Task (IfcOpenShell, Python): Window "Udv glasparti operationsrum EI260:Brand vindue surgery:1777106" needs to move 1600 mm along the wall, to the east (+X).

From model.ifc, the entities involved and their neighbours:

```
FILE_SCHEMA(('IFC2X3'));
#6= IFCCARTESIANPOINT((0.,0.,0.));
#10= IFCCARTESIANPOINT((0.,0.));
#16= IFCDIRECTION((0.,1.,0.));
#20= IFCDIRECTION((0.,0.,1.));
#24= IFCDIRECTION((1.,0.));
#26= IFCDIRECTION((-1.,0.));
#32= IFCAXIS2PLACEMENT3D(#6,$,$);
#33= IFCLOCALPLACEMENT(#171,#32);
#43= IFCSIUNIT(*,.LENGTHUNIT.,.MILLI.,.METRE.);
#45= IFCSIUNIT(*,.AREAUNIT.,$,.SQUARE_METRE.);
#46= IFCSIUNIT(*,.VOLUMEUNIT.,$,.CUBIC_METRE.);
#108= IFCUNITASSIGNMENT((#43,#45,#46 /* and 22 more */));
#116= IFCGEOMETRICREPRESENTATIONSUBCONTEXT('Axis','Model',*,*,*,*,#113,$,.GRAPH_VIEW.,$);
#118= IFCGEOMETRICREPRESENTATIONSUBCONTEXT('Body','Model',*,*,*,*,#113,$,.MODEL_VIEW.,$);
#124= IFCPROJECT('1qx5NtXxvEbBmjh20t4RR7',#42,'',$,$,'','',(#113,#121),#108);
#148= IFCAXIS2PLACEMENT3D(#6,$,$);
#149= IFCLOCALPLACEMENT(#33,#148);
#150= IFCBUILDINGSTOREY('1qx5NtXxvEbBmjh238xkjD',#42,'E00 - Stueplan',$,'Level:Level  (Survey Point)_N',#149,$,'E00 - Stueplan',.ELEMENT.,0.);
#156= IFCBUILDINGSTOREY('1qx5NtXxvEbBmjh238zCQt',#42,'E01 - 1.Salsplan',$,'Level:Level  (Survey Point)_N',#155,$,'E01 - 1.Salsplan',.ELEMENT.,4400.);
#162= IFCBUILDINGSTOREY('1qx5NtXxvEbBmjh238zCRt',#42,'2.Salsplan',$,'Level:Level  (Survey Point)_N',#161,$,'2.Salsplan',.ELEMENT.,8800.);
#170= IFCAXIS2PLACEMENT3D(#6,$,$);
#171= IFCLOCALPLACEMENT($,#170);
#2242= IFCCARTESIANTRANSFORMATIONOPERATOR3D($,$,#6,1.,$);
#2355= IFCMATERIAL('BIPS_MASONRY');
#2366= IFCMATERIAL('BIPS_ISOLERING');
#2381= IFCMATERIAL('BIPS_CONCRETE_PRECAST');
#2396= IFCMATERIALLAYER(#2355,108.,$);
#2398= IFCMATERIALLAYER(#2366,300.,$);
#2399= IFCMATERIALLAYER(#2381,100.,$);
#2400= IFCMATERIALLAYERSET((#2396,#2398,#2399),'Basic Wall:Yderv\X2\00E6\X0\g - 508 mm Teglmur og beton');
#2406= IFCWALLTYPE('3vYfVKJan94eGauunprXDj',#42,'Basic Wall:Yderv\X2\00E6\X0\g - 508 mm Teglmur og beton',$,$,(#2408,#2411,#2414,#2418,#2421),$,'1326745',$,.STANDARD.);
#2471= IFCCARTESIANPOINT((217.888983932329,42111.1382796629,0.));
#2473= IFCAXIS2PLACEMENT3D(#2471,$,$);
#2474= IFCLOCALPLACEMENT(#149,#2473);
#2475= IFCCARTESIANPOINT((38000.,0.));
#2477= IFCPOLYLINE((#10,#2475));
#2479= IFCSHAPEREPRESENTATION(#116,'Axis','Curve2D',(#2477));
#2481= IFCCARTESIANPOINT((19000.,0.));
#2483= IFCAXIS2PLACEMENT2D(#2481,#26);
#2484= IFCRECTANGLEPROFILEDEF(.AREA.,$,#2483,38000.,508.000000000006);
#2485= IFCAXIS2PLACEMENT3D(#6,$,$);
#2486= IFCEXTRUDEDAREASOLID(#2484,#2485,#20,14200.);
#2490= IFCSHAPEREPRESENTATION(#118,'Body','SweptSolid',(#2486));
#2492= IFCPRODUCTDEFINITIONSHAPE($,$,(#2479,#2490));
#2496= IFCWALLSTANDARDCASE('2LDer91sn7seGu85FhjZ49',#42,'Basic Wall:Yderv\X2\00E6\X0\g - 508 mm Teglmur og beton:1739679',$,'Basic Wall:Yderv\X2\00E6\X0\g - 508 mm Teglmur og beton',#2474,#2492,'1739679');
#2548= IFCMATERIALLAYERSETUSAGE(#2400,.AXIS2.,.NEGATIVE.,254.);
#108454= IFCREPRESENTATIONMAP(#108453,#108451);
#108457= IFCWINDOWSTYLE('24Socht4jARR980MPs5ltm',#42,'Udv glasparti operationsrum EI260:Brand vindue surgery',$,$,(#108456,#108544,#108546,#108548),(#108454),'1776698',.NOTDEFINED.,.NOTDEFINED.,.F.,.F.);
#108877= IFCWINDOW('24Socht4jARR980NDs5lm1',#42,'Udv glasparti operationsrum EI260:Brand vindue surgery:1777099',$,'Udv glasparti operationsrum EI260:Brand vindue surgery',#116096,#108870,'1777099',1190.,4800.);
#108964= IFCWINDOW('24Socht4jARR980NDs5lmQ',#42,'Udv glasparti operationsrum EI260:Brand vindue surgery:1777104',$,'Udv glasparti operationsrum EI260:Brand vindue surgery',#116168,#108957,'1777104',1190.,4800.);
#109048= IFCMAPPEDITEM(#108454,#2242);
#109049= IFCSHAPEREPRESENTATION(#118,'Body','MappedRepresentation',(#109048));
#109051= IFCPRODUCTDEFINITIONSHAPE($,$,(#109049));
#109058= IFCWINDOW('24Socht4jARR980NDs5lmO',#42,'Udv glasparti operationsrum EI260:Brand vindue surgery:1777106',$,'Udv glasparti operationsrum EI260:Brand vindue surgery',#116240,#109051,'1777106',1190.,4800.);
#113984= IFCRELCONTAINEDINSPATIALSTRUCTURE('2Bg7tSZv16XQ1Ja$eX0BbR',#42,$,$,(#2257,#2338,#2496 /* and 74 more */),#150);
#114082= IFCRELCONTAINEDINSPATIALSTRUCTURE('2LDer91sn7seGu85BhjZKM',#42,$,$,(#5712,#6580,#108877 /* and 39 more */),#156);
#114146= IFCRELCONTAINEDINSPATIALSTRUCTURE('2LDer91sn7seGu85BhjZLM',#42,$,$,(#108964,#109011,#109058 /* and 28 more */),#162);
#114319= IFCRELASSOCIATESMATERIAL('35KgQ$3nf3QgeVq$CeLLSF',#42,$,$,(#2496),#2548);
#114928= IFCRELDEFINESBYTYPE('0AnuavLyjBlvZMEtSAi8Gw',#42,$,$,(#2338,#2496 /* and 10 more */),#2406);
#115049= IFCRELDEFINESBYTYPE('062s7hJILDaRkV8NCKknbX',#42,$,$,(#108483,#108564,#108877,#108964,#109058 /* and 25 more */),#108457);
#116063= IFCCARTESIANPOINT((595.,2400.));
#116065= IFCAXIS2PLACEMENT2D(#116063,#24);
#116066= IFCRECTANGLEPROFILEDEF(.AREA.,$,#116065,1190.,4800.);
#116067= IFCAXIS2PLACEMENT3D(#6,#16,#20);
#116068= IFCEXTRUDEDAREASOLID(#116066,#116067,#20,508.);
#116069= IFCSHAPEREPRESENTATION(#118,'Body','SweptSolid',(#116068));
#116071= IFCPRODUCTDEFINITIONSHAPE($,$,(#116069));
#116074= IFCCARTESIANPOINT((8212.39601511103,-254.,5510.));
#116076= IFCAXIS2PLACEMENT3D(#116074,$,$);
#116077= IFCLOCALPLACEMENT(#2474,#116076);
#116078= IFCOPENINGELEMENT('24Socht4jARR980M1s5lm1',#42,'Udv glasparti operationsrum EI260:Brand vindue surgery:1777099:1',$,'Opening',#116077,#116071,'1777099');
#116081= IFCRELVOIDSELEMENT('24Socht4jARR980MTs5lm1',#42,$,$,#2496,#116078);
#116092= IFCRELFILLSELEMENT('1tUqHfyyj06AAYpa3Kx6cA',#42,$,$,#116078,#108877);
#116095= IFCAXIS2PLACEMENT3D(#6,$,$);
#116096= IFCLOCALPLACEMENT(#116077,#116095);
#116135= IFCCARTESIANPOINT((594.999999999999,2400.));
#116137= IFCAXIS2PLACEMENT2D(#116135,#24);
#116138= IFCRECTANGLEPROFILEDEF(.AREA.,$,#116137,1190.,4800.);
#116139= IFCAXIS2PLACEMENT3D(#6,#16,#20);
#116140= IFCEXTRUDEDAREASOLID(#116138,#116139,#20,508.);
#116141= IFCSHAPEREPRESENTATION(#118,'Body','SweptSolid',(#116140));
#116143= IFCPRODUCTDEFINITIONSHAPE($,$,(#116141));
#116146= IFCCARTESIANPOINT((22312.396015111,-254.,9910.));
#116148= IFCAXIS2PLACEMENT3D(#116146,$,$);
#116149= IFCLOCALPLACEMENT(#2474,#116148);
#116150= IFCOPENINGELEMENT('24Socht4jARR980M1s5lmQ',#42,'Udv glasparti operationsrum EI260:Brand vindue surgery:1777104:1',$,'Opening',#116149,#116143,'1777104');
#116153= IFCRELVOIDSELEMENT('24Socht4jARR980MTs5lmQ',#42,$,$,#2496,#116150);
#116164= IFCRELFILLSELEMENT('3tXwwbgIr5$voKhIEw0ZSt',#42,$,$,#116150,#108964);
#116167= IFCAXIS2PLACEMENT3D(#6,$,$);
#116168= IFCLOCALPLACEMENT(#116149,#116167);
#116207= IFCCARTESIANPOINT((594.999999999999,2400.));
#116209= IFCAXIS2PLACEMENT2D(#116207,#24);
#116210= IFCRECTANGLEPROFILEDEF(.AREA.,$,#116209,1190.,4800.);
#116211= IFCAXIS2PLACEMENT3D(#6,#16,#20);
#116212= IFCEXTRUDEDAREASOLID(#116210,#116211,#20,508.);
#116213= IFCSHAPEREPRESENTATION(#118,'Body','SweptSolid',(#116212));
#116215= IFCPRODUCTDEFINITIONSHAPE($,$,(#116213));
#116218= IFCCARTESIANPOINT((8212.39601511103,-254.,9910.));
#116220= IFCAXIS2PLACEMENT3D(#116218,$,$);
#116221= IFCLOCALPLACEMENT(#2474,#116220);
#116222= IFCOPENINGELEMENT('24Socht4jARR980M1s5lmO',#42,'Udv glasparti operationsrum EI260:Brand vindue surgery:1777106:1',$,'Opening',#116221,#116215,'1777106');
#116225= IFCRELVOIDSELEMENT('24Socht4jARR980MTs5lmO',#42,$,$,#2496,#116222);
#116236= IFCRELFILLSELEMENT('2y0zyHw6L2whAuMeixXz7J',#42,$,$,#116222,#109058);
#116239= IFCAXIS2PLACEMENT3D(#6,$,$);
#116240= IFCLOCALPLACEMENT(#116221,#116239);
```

```python
import ifcopenshell
import ifcopenshell.api.geometry
import ifcopenshell.util.placement

model = ifcopenshell.open("model.ifc")

window = model.by_id(109058)
opening = window.FillsVoids[0].RelatingOpeningElement
wall = opening.VoidsElements[0].RelatingBuildingElement

wall_matrix = ifcopenshell.util.placement.get_local_placement(wall.ObjectPlacement)
shift = wall_matrix[:3, 0] * 1600.0
before = ifcopenshell.util.placement.get_local_placement(window.ObjectPlacement)[:3, 3].copy()

# The window is placed relative to its opening, so it follows when the opening moves.
matrix = ifcopenshell.util.placement.get_local_placement(opening.ObjectPlacement)
matrix[:3, 3] += shift
ifcopenshell.api.geometry.edit_object_placement(
    model, product=opening, matrix=matrix, is_si=False, should_transform_children=True
)

after = ifcopenshell.util.placement.get_local_placement(window.ObjectPlacement)[:3, 3]
print("window moved by", (after - before).round(3) + 0.0)

model.write("model_rev.ifc")
```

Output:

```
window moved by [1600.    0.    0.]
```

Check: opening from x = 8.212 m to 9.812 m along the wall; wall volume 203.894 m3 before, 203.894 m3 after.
